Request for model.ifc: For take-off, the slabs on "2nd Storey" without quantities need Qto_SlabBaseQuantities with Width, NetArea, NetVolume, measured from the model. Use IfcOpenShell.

First a look at what the model holds.

```python
import ifcopenshell
import ifcopenshell.util.element
import ifcopenshell.util.unit

model = ifcopenshell.open("model.ifc")
print(model.schema)
for unit_type in ("LENGTHUNIT", "AREAUNIT", "VOLUMEUNIT"):
    print(unit_type, ifcopenshell.util.unit.calculate_unit_scale(model, unit_type))
storey = next(s for s in model.by_type("IfcBuildingStorey") if s.Name == "2nd Storey")
slabs = [e for e in ifcopenshell.util.element.get_decomposition(storey) if e.is_a("IfcSlab")]
for e in sorted(slabs, key=lambda e: e.id()):
    print(e.id(), e.is_a(), e.Name, list(ifcopenshell.util.element.get_psets(e, qtos_only=True)), sep=" | ")
```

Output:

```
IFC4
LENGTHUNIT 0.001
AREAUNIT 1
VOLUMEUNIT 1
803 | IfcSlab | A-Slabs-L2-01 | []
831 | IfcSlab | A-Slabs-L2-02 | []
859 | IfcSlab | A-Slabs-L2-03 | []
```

```python
import ifcopenshell
import ifcopenshell.api.pset
import ifcopenshell.geom
import ifcopenshell.util.element
import ifcopenshell.util.shape
import ifcopenshell.util.unit

model = ifcopenshell.open("model.ifc")
unit_scale = ifcopenshell.util.unit.calculate_unit_scale(model)
area_scale = ifcopenshell.util.unit.calculate_unit_scale(model, "AREAUNIT")
volume_scale = ifcopenshell.util.unit.calculate_unit_scale(model, "VOLUMEUNIT")
settings = ifcopenshell.geom.settings()

storey = next(s for s in model.by_type("IfcBuildingStorey") if s.Name == "2nd Storey")
slabs = [e for e in ifcopenshell.util.element.get_decomposition(storey) if e.is_a("IfcSlab")]

for e in sorted(slabs, key=lambda e: e.id()):
    if ifcopenshell.util.element.get_psets(e, qtos_only=True, should_inherit=False):
        continue
    # Geometry comes back in metres, in the element's own axes.
    shape = ifcopenshell.geom.create_shape(settings, e)
    values = {
        "Width": ifcopenshell.util.shape.get_z(shape.geometry) / unit_scale,
        "NetArea": ifcopenshell.util.shape.get_footprint_area(shape.geometry) / area_scale,
        "NetVolume": ifcopenshell.util.shape.get_volume(shape.geometry) / volume_scale,
    }
    qto = ifcopenshell.api.pset.add_qto(model, product=e, name="Qto_SlabBaseQuantities")
    ifcopenshell.api.pset.edit_qto(model, qto=qto, properties=values)
    print(e.id(), {k: round(v, 3) for k, v in values.items()})

model.write("model_edited.ifc")
```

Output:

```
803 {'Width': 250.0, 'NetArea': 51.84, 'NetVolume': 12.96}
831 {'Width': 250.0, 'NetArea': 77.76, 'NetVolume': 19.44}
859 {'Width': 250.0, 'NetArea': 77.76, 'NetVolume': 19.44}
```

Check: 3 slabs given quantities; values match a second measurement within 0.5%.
